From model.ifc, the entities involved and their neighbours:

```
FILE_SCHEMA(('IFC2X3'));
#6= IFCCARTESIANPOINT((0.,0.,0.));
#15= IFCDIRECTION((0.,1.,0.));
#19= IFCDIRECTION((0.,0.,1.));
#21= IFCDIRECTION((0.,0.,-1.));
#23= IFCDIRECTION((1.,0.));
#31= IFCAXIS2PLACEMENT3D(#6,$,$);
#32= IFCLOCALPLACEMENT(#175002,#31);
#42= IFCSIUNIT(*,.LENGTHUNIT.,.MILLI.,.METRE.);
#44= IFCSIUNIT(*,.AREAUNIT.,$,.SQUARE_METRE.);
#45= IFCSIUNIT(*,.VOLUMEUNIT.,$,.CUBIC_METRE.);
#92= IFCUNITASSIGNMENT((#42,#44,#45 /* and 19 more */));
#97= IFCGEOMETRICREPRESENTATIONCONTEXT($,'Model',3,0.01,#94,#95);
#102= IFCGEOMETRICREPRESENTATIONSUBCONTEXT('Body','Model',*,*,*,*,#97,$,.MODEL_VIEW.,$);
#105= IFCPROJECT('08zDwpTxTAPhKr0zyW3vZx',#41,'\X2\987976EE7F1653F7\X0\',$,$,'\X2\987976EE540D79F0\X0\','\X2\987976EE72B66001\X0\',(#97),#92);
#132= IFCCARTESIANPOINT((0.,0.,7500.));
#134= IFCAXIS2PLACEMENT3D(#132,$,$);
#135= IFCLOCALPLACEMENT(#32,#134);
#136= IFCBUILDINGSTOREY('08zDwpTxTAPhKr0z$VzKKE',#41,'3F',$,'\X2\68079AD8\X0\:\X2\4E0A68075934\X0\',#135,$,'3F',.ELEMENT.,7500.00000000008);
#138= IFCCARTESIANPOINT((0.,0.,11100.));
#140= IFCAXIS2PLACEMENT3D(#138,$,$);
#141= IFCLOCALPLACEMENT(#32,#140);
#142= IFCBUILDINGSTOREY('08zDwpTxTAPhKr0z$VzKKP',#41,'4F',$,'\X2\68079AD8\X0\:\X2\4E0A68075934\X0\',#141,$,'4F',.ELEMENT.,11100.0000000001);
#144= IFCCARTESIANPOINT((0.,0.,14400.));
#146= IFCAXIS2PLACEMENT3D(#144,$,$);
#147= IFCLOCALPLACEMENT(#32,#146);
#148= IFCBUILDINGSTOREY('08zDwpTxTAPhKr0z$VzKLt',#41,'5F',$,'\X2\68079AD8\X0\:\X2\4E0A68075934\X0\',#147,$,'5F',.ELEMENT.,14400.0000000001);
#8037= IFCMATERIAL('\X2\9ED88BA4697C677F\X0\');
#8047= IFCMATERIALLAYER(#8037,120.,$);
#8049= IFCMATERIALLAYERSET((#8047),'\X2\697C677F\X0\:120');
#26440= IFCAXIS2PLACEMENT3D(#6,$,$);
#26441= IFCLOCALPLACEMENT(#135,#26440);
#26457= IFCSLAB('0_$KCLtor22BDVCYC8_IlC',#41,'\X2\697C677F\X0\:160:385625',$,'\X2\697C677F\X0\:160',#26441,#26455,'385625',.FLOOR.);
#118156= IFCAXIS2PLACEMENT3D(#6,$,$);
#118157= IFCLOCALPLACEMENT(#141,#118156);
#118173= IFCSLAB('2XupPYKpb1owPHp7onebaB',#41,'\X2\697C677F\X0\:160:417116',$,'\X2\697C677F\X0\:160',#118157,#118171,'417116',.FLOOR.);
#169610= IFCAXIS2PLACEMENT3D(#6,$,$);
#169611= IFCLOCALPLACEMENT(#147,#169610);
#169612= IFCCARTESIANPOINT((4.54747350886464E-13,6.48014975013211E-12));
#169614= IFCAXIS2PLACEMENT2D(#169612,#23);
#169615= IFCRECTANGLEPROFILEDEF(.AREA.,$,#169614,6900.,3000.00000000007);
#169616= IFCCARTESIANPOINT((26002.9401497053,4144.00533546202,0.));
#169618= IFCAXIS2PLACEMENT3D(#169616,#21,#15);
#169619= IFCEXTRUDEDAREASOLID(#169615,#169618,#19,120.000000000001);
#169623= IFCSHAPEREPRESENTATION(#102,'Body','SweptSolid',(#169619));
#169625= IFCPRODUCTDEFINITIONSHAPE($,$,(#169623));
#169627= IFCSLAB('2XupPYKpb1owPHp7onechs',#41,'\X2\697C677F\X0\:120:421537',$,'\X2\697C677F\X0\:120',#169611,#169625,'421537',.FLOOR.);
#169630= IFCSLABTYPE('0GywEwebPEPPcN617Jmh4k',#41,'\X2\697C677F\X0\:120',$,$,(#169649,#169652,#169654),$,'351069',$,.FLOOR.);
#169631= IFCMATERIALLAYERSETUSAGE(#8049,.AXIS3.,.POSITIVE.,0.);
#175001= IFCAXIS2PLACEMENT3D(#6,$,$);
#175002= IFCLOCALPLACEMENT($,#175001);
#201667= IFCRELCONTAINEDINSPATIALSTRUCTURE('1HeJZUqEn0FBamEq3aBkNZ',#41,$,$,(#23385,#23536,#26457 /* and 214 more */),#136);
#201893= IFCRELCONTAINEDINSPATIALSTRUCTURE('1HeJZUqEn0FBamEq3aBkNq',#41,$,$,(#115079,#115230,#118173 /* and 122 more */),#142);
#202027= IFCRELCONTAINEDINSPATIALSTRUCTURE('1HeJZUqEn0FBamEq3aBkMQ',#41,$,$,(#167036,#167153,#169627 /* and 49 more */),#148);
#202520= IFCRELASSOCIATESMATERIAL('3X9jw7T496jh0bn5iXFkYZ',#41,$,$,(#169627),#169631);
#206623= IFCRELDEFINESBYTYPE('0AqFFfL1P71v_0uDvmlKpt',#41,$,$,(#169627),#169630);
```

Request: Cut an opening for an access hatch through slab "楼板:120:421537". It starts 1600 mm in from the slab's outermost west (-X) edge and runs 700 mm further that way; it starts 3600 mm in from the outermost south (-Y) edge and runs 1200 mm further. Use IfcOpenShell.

```python
import numpy as np
import ifcopenshell
import ifcopenshell.api.feature
import ifcopenshell.api.geometry
import ifcopenshell.api.root
import ifcopenshell.geom
import ifcopenshell.util.placement
import ifcopenshell.util.representation
import ifcopenshell.util.shape
import ifcopenshell.util.unit

model = ifcopenshell.open("model.ifc")
unit_scale = ifcopenshell.util.unit.calculate_unit_scale(model)
settings = ifcopenshell.geom.settings()


def volume(element):
    """Net volume in cubic metres, openings subtracted."""
    shape = ifcopenshell.geom.create_shape(settings, element)
    return ifcopenshell.util.shape.get_volume(shape.geometry)


slab = model.by_guid("2XupPYKpb1owPHp7onechs")
before = volume(slab)

# Extent in the slab's own axes, in metres. The edges named are its -X and -Y sides.
slab_shape = ifcopenshell.geom.create_shape(settings, slab)
vertices = ifcopenshell.util.shape.get_vertices(slab_shape.geometry)
x_min, y_min, bottom = vertices.min(axis=0)
top = vertices[:, 2].max()

opening = ifcopenshell.api.root.create_entity(model, ifc_class="IfcOpeningElement", name="Access hatch opening")
context = ifcopenshell.util.representation.get_context(model, "Model", "Body", "MODEL_VIEW")
width, depth = 0.7, 1.2
outline = [(0.0, 0.0), (width, 0.0), (width, depth), (0.0, depth), (0.0, 0.0)]
# Overshoot both faces by 50 mm so the cut is clean.
shape = ifcopenshell.api.geometry.add_slab_representation(
    model, context=context, depth=top - bottom + 0.1, polyline=outline
)
ifcopenshell.api.geometry.assign_representation(model, product=opening, representation=shape)

matrix = ifcopenshell.util.placement.get_local_placement(slab.ObjectPlacement)
matrix[:, 3] = matrix @ np.append(np.array([x_min + 1.6, y_min + 3.6, bottom - 0.05]) / unit_scale, 1.0)
ifcopenshell.api.geometry.edit_object_placement(model, product=opening, matrix=matrix, is_si=False)
ifcopenshell.api.feature.add_feature(model, feature=opening, element=slab)

after = volume(slab)

print(f"slab volume {before:.3f} -> {after:.3f} m3")

model.write("model-out.ifc")
```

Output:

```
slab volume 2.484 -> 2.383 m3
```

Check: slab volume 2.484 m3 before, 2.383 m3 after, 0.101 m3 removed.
